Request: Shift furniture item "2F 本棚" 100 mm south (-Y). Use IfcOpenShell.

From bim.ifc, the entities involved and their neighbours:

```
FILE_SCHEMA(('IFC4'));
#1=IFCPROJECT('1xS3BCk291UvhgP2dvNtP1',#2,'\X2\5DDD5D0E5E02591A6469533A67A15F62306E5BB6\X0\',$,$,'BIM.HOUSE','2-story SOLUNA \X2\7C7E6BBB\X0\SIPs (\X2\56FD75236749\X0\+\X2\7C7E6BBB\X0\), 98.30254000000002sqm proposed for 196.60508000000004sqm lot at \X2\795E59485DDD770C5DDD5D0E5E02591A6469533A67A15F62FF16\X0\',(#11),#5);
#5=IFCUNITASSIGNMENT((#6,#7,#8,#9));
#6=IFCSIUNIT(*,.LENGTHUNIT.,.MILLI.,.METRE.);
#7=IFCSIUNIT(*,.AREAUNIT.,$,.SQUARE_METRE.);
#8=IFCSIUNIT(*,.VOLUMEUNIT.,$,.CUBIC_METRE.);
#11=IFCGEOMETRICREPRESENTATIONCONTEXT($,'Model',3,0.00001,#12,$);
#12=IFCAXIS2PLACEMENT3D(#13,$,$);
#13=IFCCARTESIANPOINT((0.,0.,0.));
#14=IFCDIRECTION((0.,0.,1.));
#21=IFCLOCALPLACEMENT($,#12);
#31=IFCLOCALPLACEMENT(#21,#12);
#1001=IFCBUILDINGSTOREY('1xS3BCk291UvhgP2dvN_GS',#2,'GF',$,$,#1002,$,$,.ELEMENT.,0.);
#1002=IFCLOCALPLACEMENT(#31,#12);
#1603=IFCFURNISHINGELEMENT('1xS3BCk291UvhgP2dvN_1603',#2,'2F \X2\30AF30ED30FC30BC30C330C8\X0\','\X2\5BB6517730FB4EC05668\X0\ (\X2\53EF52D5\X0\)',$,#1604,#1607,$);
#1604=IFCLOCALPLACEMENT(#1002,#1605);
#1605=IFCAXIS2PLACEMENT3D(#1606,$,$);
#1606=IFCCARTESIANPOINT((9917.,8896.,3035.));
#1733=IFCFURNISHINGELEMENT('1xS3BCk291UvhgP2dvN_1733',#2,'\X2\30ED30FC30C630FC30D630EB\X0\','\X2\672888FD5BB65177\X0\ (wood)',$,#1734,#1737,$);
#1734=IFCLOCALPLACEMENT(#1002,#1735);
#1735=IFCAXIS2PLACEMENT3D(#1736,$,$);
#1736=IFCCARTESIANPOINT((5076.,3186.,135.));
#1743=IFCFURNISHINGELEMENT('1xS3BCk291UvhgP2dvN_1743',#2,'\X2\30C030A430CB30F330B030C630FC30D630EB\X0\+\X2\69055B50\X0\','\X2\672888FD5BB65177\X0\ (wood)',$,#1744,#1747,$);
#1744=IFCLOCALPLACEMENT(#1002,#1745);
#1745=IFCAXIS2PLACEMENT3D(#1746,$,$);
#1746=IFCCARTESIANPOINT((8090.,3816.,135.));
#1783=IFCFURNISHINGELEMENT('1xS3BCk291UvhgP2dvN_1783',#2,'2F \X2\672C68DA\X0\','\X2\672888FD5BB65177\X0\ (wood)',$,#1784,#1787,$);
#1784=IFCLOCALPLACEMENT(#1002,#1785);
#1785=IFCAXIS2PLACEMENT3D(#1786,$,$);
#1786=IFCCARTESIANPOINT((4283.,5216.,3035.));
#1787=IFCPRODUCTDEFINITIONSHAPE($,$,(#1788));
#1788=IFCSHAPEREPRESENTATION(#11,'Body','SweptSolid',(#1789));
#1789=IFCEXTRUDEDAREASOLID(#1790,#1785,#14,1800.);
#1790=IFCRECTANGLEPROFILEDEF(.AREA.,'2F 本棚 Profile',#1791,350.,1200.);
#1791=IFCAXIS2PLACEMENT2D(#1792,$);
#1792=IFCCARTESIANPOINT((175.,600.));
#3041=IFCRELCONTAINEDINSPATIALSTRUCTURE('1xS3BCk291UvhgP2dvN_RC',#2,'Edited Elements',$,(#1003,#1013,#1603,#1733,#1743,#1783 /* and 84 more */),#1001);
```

```python
import ifcopenshell
import ifcopenshell.api.geometry
import ifcopenshell.util.placement
import ifcopenshell.util.unit

model = ifcopenshell.open("bim.ifc")
unit_scale = ifcopenshell.util.unit.calculate_unit_scale(model)

item = model.by_guid("1xS3BCk291UvhgP2dvN_1783")
matrix = ifcopenshell.util.placement.get_local_placement(item.ObjectPlacement)
matrix[1, 3] -= 0.1 / unit_scale
ifcopenshell.api.geometry.edit_object_placement(model, product=item, matrix=matrix, is_si=False)

print(ifcopenshell.util.placement.get_local_placement(item.ObjectPlacement).round(3) + 0.0)

model.write("bim_edited.ifc")
```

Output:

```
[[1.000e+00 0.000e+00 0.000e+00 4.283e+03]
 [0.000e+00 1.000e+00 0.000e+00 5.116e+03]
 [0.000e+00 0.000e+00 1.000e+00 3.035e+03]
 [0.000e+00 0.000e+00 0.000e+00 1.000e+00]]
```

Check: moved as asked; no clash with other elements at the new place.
